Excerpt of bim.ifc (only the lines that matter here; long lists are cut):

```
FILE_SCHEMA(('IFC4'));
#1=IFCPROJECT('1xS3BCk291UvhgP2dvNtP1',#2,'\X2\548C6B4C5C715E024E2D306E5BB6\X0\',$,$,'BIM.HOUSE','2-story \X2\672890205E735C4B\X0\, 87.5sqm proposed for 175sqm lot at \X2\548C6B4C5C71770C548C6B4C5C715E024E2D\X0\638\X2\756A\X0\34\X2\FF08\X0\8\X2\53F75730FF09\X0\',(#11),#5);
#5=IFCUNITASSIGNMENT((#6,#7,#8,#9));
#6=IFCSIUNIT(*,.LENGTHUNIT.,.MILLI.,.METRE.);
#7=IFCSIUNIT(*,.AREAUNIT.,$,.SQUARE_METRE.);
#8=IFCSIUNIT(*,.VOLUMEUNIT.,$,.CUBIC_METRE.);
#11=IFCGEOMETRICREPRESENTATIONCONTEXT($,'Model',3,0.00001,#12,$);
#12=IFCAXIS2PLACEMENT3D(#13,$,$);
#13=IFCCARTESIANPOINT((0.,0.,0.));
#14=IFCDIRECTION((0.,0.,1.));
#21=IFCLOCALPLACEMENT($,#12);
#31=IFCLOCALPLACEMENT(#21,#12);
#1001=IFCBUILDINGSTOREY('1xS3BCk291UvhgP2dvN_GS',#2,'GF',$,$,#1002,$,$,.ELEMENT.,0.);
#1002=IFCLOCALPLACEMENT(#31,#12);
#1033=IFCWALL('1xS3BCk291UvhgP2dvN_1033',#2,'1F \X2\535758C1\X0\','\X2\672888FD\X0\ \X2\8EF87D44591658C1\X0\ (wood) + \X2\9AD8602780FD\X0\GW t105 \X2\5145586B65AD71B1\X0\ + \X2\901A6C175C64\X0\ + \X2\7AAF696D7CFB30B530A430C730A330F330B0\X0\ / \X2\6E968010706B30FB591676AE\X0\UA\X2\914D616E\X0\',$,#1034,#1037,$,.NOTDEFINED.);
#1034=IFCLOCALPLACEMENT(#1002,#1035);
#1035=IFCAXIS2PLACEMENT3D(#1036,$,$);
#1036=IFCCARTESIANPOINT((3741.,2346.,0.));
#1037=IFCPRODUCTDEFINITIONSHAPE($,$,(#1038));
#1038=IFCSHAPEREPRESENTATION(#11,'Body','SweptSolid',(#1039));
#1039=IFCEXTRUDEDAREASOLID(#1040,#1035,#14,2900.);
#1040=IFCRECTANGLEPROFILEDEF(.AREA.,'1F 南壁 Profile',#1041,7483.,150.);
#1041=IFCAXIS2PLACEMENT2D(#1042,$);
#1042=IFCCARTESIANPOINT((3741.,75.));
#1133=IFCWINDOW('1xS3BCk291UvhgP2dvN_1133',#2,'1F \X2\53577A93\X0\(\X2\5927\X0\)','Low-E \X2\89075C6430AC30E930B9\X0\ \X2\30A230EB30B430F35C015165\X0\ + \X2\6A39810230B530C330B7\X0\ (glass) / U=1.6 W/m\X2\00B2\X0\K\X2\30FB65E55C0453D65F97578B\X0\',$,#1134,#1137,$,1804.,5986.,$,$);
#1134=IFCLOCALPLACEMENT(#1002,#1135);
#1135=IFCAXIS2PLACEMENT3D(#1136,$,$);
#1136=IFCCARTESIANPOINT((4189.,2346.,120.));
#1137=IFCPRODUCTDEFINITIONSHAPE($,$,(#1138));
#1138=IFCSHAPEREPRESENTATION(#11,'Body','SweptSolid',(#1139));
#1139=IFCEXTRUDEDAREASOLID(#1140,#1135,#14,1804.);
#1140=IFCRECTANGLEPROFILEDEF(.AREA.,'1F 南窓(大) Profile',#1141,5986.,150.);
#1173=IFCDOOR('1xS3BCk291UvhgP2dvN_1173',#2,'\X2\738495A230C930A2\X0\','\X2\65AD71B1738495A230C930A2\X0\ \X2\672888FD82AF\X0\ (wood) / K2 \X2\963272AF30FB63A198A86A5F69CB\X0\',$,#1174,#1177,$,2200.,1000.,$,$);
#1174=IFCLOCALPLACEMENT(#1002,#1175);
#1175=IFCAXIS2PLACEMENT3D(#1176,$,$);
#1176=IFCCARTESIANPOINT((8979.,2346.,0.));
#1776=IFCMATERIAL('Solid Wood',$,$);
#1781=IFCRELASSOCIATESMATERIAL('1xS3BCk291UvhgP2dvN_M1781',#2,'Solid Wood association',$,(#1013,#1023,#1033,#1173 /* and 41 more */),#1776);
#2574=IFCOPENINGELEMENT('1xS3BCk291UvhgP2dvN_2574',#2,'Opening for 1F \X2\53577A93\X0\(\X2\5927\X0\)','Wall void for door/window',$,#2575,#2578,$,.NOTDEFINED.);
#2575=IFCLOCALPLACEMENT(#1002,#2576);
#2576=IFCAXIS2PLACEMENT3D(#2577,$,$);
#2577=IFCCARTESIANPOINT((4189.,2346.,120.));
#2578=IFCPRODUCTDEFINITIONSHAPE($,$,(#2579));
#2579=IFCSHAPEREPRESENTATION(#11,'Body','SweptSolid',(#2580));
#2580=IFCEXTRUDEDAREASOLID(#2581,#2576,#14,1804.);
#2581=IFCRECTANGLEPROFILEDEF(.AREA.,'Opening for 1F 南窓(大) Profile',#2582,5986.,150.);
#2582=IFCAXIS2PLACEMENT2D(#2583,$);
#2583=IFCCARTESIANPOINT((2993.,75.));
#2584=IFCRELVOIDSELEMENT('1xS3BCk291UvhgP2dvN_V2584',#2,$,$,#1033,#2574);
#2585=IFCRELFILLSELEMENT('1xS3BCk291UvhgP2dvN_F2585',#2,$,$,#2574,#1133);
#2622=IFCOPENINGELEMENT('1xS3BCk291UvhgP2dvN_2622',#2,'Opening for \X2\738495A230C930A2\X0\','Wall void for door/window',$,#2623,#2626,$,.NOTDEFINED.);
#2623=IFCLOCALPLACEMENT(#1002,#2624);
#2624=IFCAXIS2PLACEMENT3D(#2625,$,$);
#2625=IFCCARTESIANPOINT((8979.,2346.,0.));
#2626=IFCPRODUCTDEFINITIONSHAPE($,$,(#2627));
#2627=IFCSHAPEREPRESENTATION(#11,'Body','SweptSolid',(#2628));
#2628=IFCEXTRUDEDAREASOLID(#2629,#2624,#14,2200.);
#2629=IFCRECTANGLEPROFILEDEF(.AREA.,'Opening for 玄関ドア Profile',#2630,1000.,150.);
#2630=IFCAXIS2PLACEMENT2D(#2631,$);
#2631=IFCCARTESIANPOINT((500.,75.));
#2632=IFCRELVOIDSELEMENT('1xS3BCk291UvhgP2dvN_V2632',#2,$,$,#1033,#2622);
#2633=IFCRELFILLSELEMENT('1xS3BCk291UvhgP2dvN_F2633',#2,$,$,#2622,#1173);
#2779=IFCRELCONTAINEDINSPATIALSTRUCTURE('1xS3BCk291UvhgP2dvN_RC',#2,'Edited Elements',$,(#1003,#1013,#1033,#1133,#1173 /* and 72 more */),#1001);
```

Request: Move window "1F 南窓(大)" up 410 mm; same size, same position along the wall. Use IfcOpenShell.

```python
import numpy as np
import ifcopenshell
import ifcopenshell.api.geometry
import ifcopenshell.util.placement
import ifcopenshell.util.unit

model = ifcopenshell.open("bim.ifc")
unit_scale = ifcopenshell.util.unit.calculate_unit_scale(model)

window = model.by_id(1133)
opening = window.FillsVoids[0].RelatingOpeningElement
dz = 410.0

shift = np.array([0.0, 0.0, dz])
# The window is not placed relative to its opening, so move both.
for product in (opening, window):
    matrix = ifcopenshell.util.placement.get_local_placement(product.ObjectPlacement)
    matrix[:3, 3] += shift
    ifcopenshell.api.geometry.edit_object_placement(model, product=product, matrix=matrix, is_si=False)

print(f"moved by {dz * unit_scale:+.3f} m")

model.write("bim_edited.ifc")
```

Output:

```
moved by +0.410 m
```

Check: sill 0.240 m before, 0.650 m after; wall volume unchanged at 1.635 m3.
